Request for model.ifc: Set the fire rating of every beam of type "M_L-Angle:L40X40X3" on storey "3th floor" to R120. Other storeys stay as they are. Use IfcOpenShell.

First a look at what the model holds.

```python
import ifcopenshell
import ifcopenshell.util.element

model = ifcopenshell.open("model.ifc")
print(model.schema)
storey = next(s for s in model.by_type("IfcBuildingStorey") if s.Name == "3th floor")
beams = [e for e in ifcopenshell.util.element.get_decomposition(storey) if e.is_a("IfcBeam")]
seen = {}
for e in beams:
    element_type = ifcopenshell.util.element.get_type(e)
    key = (element_type.Name if element_type != e and element_type else None, ifcopenshell.util.element.get_pset(e, "Pset_BeamCommon", "FireRating"))
    seen[key] = seen.get(key, 0) + 1
for (name, value), count in sorted(seen.items(), key=str):
    print(count, "x", name, "|", value)
```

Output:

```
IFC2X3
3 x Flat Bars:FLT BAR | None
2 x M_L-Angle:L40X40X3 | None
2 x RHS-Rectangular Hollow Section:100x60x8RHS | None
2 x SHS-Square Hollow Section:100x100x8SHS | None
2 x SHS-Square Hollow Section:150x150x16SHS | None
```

```python
import ifcopenshell
import ifcopenshell.api.pset
import ifcopenshell.util.element

model = ifcopenshell.open("model.ifc")

storey = next(s for s in model.by_type("IfcBuildingStorey") if s.Name == "3th floor")
beams = [e for e in ifcopenshell.util.element.get_decomposition(storey) if e.is_a("IfcBeam")]

count = 0
for e in beams:
    element_type = ifcopenshell.util.element.get_type(e)
    if element_type in (None, e) or element_type.Name != "M_L-Angle:L40X40X3":
        continue
    # add_pset returns the element's existing set when there is one.
    pset = ifcopenshell.api.pset.add_pset(model, product=e, name="Pset_BeamCommon")
    ifcopenshell.api.pset.edit_pset(model, pset=pset, properties={"FireRating": "R120"})
    count += 1

print(count, "beams updated")

model.write("model-out.ifc")
```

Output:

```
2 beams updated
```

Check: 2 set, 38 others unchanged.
